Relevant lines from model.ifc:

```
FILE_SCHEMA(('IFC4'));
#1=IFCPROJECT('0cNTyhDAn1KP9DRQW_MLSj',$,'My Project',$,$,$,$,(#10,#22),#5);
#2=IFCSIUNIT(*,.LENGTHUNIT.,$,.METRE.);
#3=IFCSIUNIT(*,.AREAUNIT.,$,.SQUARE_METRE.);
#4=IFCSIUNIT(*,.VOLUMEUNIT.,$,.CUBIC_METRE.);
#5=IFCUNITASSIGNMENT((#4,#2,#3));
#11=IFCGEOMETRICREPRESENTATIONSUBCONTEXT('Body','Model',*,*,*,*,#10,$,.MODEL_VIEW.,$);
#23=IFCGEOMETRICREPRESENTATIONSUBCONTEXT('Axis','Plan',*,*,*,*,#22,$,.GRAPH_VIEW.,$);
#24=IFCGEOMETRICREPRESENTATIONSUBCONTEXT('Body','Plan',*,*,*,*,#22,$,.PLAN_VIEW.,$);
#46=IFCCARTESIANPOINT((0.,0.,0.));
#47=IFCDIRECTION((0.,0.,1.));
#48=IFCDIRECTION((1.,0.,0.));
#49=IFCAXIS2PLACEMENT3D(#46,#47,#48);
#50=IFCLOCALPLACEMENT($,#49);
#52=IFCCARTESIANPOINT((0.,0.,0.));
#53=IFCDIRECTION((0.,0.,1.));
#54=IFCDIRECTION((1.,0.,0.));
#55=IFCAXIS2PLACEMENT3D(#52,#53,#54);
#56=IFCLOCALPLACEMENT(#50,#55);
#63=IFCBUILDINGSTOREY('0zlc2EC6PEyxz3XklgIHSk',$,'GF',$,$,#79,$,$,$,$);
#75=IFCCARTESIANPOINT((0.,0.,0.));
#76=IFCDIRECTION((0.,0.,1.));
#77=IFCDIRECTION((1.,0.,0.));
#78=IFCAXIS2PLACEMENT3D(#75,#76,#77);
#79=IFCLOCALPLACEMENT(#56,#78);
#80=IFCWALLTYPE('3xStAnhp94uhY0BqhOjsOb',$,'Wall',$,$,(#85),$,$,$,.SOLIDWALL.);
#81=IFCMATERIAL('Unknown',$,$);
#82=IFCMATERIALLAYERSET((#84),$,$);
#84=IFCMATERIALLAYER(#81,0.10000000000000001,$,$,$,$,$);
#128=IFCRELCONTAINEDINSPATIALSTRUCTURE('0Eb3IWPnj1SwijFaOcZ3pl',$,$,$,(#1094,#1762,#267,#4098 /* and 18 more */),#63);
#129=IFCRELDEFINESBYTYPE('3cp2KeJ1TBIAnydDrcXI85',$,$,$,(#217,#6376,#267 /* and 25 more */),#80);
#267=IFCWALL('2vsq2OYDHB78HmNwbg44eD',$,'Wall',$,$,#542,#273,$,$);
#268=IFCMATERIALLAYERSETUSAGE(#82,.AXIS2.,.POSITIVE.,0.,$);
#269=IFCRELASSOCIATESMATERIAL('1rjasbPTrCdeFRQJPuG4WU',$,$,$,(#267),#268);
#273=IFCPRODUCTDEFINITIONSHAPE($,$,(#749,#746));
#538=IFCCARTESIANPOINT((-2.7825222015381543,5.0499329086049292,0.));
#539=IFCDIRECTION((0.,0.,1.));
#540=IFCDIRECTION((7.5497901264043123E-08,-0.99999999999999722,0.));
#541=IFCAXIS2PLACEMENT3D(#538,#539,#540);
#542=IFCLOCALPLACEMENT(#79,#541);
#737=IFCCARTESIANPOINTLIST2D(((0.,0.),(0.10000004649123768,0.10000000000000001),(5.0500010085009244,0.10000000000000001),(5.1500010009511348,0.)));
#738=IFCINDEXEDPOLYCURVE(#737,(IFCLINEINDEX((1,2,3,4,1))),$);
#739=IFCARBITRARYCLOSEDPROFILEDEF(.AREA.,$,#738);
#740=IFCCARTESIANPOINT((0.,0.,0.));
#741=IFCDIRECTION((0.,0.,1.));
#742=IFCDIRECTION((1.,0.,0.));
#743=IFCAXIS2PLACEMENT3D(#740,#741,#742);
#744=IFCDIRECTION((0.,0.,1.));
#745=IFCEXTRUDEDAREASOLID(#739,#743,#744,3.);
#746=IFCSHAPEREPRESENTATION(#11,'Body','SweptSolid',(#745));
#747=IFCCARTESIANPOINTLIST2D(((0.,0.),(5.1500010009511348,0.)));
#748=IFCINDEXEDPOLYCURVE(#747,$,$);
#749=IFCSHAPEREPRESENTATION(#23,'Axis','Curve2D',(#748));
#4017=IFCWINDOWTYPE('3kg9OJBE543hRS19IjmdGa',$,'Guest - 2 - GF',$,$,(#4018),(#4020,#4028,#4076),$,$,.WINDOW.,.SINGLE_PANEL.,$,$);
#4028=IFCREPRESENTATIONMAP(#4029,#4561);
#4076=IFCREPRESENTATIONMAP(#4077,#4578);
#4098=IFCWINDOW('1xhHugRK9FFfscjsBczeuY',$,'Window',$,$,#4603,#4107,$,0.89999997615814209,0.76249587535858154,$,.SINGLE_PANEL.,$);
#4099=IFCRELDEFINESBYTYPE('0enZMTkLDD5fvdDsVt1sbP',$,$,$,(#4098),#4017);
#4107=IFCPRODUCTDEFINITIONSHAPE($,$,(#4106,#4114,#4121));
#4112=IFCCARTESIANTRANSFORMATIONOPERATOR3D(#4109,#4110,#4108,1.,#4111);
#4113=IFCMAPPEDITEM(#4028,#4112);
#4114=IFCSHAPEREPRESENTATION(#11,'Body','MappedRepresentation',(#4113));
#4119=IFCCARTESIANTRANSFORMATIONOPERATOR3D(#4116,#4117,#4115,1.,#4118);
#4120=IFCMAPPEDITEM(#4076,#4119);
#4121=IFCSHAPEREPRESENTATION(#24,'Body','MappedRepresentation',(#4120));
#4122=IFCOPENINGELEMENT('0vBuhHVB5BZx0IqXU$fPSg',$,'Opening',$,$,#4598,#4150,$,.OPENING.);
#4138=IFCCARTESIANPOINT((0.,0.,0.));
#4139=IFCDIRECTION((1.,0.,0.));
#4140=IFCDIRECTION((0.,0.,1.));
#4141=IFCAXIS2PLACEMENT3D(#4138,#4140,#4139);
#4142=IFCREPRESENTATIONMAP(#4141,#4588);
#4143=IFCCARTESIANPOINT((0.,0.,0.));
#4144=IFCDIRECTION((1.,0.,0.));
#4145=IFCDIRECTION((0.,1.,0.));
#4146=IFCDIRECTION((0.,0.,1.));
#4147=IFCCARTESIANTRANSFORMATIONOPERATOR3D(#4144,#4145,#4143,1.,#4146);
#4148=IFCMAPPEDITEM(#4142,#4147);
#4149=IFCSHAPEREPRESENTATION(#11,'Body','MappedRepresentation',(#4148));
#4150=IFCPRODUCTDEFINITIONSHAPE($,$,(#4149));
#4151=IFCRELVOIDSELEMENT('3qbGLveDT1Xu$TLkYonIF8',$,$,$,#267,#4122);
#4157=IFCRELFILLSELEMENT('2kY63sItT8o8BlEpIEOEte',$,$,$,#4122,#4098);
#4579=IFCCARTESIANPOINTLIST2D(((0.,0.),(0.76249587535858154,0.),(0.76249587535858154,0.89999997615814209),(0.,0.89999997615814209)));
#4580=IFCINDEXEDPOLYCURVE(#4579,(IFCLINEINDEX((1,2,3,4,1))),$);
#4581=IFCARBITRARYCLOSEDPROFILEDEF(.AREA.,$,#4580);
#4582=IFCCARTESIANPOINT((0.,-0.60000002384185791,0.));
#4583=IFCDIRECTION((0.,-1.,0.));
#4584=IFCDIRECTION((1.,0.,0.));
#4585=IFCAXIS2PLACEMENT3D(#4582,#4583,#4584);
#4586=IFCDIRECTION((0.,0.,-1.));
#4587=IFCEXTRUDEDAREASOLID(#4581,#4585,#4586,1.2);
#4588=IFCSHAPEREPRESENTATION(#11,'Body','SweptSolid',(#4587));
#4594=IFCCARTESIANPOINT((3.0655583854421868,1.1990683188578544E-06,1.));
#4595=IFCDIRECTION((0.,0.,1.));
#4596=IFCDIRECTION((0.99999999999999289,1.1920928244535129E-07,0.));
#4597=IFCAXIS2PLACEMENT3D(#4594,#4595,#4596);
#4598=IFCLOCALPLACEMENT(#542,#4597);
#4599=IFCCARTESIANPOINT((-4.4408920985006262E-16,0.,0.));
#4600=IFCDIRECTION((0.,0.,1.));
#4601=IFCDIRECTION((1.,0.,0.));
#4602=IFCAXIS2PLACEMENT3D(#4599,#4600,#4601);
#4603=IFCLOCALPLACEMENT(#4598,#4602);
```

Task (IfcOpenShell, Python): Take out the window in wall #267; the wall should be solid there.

```python
import ifcopenshell
import ifcopenshell.api.feature
import ifcopenshell.api.root
import ifcopenshell.geom
import ifcopenshell.util.shape

model = ifcopenshell.open("model.ifc")
settings = ifcopenshell.geom.settings()


def volume(element):
    """Net volume in cubic metres, openings subtracted."""
    shape = ifcopenshell.geom.create_shape(settings, element)
    return ifcopenshell.util.shape.get_volume(shape.geometry)


window = model.by_id(4098)
opening = window.FillsVoids[0].RelatingOpeningElement
wall = opening.VoidsElements[0].RelatingBuildingElement
before = volume(wall)

ifcopenshell.api.root.remove_product(model, product=window)
ifcopenshell.api.feature.remove_feature(model, feature=opening)

after = volume(wall)

print(f"wall volume {before:.3f} -> {after:.3f} m3")

model.write("model-out.ifc")
```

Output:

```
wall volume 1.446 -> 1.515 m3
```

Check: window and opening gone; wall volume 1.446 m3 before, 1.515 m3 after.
